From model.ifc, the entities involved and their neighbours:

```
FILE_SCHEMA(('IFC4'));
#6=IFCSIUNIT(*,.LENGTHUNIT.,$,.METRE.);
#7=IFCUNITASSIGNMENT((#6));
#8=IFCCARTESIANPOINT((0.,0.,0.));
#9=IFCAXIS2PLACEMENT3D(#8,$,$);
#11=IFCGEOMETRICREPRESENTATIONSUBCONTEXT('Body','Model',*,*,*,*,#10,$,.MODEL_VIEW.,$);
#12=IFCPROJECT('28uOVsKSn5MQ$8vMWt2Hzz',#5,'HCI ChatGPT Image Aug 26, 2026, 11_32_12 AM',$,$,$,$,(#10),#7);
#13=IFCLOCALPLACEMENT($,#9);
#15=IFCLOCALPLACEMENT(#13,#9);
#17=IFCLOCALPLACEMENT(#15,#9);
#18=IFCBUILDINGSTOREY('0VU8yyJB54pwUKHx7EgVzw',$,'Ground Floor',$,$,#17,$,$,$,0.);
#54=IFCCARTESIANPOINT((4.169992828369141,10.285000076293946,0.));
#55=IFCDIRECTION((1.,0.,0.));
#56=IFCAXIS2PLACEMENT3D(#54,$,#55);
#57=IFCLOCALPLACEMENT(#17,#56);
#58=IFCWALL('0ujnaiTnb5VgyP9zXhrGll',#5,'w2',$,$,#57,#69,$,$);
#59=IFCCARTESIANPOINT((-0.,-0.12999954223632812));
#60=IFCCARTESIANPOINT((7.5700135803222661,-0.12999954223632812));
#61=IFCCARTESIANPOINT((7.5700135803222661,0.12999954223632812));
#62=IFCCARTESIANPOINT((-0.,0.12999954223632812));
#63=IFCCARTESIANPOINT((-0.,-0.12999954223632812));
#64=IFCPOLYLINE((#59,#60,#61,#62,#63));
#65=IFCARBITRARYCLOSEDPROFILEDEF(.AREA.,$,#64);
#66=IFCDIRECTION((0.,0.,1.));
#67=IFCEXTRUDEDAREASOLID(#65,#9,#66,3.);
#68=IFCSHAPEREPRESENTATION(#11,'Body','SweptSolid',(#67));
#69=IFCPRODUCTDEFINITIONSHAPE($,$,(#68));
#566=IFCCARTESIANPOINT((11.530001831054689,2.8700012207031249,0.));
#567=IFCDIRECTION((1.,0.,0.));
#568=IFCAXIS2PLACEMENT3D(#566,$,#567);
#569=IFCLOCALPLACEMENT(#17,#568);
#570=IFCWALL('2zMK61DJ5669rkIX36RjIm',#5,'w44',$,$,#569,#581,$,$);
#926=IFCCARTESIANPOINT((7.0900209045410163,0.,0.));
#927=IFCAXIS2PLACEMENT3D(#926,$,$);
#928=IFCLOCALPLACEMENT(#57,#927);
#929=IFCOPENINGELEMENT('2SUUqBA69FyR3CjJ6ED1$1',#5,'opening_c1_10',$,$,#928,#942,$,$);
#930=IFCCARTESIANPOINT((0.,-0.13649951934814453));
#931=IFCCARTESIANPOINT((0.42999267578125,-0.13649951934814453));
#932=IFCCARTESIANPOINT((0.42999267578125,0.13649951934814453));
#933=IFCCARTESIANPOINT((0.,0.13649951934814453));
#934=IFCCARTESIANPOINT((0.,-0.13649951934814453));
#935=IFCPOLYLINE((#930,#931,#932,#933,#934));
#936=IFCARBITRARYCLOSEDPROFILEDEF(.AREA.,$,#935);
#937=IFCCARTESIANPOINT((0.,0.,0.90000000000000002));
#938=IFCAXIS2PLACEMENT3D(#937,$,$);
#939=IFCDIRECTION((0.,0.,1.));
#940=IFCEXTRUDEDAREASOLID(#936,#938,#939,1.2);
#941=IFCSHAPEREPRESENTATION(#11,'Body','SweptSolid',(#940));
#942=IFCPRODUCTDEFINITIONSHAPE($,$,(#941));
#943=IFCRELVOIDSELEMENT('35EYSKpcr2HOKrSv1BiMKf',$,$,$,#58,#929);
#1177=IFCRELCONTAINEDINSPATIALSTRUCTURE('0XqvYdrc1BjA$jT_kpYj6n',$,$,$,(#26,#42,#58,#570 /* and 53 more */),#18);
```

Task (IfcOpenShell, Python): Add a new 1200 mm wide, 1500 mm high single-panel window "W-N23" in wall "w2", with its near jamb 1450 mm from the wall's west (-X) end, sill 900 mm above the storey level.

```python
import numpy as np
import ifcopenshell
import ifcopenshell.api.feature
import ifcopenshell.api.geometry
import ifcopenshell.api.root
import ifcopenshell.api.spatial
import ifcopenshell.geom
import ifcopenshell.util.element
import ifcopenshell.util.placement
import ifcopenshell.util.representation
import ifcopenshell.util.shape
import ifcopenshell.util.unit

model = ifcopenshell.open("model.ifc")
unit_scale = ifcopenshell.util.unit.calculate_unit_scale(model)
settings = ifcopenshell.geom.settings()


def volume(element):
    """Net volume in cubic metres, openings subtracted."""
    shape = ifcopenshell.geom.create_shape(settings, element)
    return ifcopenshell.util.shape.get_volume(shape.geometry)


wall = model.by_guid("0ujnaiTnb5VgyP9zXhrGll")
storey = ifcopenshell.util.element.get_container(wall, ifc_class="IfcBuildingStorey")
context = ifcopenshell.util.representation.get_context(model, "Model", "Body", "MODEL_VIEW")
before = volume(wall)

width, height, from_end, sill = 1.2, 1.5, 1.45, 0.9  # metres

# The wall runs along its own X axis, and the end named is its -X end.
wall_shape = ifcopenshell.geom.create_shape(settings, wall)
x, y, z = ifcopenshell.util.shape.get_vertices(wall_shape.geometry).T
start = x.min() + from_end
face, thickness = float(y.min()), float(y.max() - y.min())
wall_matrix = ifcopenshell.util.placement.get_local_placement(wall.ObjectPlacement)
level = ifcopenshell.util.placement.get_local_placement(storey.ObjectPlacement)[2, 3]


def in_wall(x, y):
    """Placement at x, y metres in the wall's axes, at sill height."""
    matrix = wall_matrix.copy()
    matrix[:, 3] = wall_matrix @ np.array([x / unit_scale, y / unit_scale, 0.0, 1.0])
    matrix[2, 3] = level + sill / unit_scale
    return matrix


# Opening: a box that overshoots both wall faces by 50 mm.
opening = ifcopenshell.api.root.create_entity(model, ifc_class="IfcOpeningElement", predefined_type="OPENING")
box = ifcopenshell.api.geometry.add_wall_representation(
    model, context=context, length=width, height=height, thickness=thickness + 0.1
)
ifcopenshell.api.geometry.assign_representation(model, product=opening, representation=box)
ifcopenshell.api.geometry.edit_object_placement(model, product=opening, matrix=in_wall(start, face - 0.05), is_si=False)
ifcopenshell.api.feature.add_feature(model, feature=opening, element=wall)

window = ifcopenshell.api.root.create_entity(model, ifc_class="IfcWindow", name="W-N23", predefined_type="WINDOW")
window.OverallWidth, window.OverallHeight = width / unit_scale, height / unit_scale
window.PartitioningType = "SINGLE_PANEL"
body = ifcopenshell.api.geometry.add_window_representation(
    model,
    context=context,
    overall_width=window.OverallWidth,
    overall_height=window.OverallHeight,
    partition_type="SINGLE_PANEL",
)
ifcopenshell.api.geometry.assign_representation(model, product=window, representation=body)
ifcopenshell.api.spatial.assign_container(model, products=[window], relating_structure=storey)
ifcopenshell.api.feature.add_filling(model, opening=opening, element=window)

# Centre the window in the wall's thickness.
ifcopenshell.api.geometry.edit_object_placement(model, product=window, matrix=in_wall(start, face), is_si=False)
window_shape = ifcopenshell.geom.create_shape(settings, window)
depth = ifcopenshell.util.shape.get_vertices(window_shape.geometry)[:, 1]
offset = face + thickness / 2 - (depth.min() + depth.max()) / 2
ifcopenshell.api.geometry.edit_object_placement(model, product=window, matrix=in_wall(start, offset), is_si=False)

after = volume(wall)

print(f"wall volume {before:.3f} -> {after:.3f} m3")

model.write("model_v2.ifc")
```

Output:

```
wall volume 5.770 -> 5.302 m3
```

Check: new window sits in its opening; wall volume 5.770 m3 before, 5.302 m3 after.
